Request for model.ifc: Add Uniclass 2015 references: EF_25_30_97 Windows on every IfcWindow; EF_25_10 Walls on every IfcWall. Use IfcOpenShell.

First a look at what the model holds.

```python
import ifcopenshell

model = ifcopenshell.open("model.ifc")
print(model.schema)
print("classifications:", [c.Name for c in model.by_type("IfcClassification")])
for ifc_class in ("IfcDoor", "IfcRoof", "IfcStair", "IfcWall", "IfcWindow"):
    print(ifc_class, len(model.by_type(ifc_class)))
```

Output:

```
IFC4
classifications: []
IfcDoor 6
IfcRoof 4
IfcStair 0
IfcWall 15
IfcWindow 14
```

```python
import ifcopenshell
import ifcopenshell.api.classification

model = ifcopenshell.open("model.ifc")

system = ifcopenshell.api.classification.add_classification(model, classification="Uniclass 2015")

codes = {
    "IfcWindow": ("EF_25_30_97", "Windows"),
    "IfcWall": ("EF_25_10", "Walls"),
}
for ifc_class, (code, name) in codes.items():
    products = model.by_type(ifc_class)
    ifcopenshell.api.classification.add_reference(
        model, products=products, classification=system, identification=code, name=name
    )
    print(code, len(products))

model.write("model_rev.ifc")
```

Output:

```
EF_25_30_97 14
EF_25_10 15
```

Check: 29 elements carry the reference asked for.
